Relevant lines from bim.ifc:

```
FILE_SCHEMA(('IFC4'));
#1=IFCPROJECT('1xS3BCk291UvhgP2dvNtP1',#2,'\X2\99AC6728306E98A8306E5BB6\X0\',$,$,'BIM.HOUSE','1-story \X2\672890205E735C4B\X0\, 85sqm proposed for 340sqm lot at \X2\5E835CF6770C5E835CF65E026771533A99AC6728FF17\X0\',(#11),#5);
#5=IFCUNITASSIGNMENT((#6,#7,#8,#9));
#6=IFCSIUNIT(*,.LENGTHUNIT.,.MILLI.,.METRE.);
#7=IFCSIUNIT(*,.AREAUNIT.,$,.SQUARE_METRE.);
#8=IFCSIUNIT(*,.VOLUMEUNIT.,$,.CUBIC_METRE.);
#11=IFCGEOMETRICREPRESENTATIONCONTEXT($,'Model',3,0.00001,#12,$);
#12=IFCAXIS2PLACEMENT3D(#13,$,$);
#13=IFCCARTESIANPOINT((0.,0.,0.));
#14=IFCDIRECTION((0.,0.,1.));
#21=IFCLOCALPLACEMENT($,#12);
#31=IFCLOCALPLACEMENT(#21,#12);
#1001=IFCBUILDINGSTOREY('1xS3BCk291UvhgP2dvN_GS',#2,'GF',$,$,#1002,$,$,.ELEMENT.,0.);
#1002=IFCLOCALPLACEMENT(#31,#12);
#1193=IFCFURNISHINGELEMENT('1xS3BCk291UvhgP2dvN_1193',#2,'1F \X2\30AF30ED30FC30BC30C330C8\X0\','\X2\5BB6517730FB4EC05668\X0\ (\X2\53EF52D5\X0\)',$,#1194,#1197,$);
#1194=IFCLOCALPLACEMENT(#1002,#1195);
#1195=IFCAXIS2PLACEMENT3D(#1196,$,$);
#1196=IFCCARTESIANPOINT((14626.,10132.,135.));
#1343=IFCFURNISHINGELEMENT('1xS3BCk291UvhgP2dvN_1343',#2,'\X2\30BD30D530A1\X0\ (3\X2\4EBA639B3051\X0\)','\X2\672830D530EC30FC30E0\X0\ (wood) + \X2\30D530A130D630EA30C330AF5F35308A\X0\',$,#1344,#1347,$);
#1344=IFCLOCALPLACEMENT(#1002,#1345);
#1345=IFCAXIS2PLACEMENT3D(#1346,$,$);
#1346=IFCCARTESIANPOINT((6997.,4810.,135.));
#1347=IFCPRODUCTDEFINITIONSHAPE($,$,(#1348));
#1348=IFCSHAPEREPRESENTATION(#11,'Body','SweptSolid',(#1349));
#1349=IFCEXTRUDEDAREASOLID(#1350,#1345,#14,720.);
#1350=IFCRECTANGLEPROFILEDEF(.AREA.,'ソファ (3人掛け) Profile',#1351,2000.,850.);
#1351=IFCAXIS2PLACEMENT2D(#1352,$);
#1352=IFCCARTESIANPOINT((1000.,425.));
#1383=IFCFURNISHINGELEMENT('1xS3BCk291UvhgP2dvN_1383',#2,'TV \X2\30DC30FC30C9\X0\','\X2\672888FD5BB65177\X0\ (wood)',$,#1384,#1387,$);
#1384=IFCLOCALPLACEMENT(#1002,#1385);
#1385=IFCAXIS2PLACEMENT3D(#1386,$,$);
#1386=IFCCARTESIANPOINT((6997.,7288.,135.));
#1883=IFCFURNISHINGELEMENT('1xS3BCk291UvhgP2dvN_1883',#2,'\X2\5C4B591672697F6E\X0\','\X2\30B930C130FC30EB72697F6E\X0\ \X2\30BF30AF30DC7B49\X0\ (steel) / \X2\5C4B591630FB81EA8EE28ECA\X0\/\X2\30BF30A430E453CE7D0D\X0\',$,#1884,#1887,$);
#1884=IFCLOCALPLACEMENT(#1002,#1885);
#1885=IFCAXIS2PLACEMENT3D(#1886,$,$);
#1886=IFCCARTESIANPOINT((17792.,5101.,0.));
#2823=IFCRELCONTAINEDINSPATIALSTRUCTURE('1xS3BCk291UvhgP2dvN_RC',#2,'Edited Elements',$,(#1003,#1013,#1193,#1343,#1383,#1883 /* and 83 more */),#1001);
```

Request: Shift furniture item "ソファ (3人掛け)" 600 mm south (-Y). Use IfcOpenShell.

```python
import ifcopenshell
import ifcopenshell.api.geometry
import ifcopenshell.util.placement

model = ifcopenshell.open("bim.ifc")

item = model.by_guid("1xS3BCk291UvhgP2dvN_1343")
matrix = ifcopenshell.util.placement.get_local_placement(item.ObjectPlacement)
matrix[1, 3] -= 600.0
ifcopenshell.api.geometry.edit_object_placement(model, product=item, matrix=matrix, is_si=False)

print(ifcopenshell.util.placement.get_local_placement(item.ObjectPlacement).round(3) + 0.0)

model.write("bim_updated.ifc")
```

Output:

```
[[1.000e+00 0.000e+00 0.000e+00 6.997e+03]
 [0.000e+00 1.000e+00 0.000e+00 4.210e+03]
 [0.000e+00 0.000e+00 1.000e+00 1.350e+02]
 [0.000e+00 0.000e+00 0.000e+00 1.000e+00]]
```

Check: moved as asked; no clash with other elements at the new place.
